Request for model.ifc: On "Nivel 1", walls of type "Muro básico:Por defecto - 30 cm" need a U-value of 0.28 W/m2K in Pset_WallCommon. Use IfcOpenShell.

First a look at what the model holds.

```python
import ifcopenshell
import ifcopenshell.util.element

model = ifcopenshell.open("model.ifc")
print(model.schema)
storey = next(s for s in model.by_type("IfcBuildingStorey") if s.Name == "Nivel 1")
walls = [e for e in ifcopenshell.util.element.get_decomposition(storey) if e.is_a("IfcWall")]
seen = {}
for e in walls:
    element_type = ifcopenshell.util.element.get_type(e)
    key = (element_type.Name if element_type != e and element_type else None, ifcopenshell.util.element.get_pset(e, "Pset_WallCommon", "ThermalTransmittance"))
    seen[key] = seen.get(key, 0) + 1
for (name, value), count in sorted(seen.items(), key=str):
    print(count, "x", name, "|", value)
```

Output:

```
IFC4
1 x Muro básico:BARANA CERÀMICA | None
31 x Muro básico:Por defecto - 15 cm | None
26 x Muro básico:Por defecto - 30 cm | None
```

```python
import ifcopenshell
import ifcopenshell.api.pset
import ifcopenshell.util.element

model = ifcopenshell.open("model.ifc")

storey = next(s for s in model.by_type("IfcBuildingStorey") if s.Name == "Nivel 1")
walls = [e for e in ifcopenshell.util.element.get_decomposition(storey) if e.is_a("IfcWall")]

count = 0
for e in walls:
    element_type = ifcopenshell.util.element.get_type(e)
    if element_type in (None, e) or element_type.Name != "Muro básico:Por defecto - 30 cm":
        continue
    # add_pset returns the element's existing set when there is one.
    pset = ifcopenshell.api.pset.add_pset(model, product=e, name="Pset_WallCommon")
    ifcopenshell.api.pset.edit_pset(model, pset=pset, properties={"ThermalTransmittance": 0.28})
    count += 1

print(count, "walls updated")

model.write("model-out.ifc")
```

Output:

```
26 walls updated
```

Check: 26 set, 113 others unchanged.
